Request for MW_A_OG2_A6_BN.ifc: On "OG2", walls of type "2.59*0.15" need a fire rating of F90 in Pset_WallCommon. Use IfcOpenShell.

First a look at what the model holds.

```python
import ifcopenshell
import ifcopenshell.util.element

model = ifcopenshell.open("MW_A_OG2_A6_BN.ifc")
print(model.schema)
storey = next(s for s in model.by_type("IfcBuildingStorey") if s.Name == "OG2")
walls = [e for e in ifcopenshell.util.element.get_decomposition(storey) if e.is_a("IfcWall")]
seen = {}
for e in walls:
    element_type = ifcopenshell.util.element.get_type(e)
    key = (element_type.Name if element_type != e and element_type else None, ifcopenshell.util.element.get_pset(e, "Pset_WallCommon", "FireRating"))
    seen[key] = seen.get(key, 0) + 1
for (name, value), count in sorted(seen.items(), key=str):
    print(count, "x", name, "|", value)
```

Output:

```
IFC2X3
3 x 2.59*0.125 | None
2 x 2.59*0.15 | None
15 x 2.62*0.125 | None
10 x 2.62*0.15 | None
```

```python
import ifcopenshell
import ifcopenshell.api.pset
import ifcopenshell.util.element

model = ifcopenshell.open("MW_A_OG2_A6_BN.ifc")

storey = next(s for s in model.by_type("IfcBuildingStorey") if s.Name == "OG2")
walls = [e for e in ifcopenshell.util.element.get_decomposition(storey) if e.is_a("IfcWall")]

count = 0
for e in walls:
    element_type = ifcopenshell.util.element.get_type(e)
    if element_type in (None, e) or element_type.Name != "2.59*0.15":
        continue
    found = ifcopenshell.util.element.get_pset(e, "Pset_WallCommon", should_inherit=False)
    if found:
        pset = model.by_id(found["id"])
        if len(ifcopenshell.util.element.get_elements_by_pset(pset)) > 1:
            pset = ifcopenshell.api.pset.unshare_pset(model, products=[e], pset=pset)[0]
    else:
        pset = ifcopenshell.api.pset.add_pset(model, product=e, name="Pset_WallCommon")
    ifcopenshell.api.pset.edit_pset(model, pset=pset, properties={"FireRating": "F90"})
    count += 1

print(count, "walls updated")

model.write("MW_A_OG2_A6_BN_rev.ifc")
```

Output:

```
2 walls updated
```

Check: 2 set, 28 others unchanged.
